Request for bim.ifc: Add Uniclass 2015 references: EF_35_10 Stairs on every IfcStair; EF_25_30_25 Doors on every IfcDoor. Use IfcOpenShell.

First a look at what the model holds.

```python
import ifcopenshell

model = ifcopenshell.open("bim.ifc")
print(model.schema)
print("classifications:", [c.Name for c in model.by_type("IfcClassification")])
for ifc_class in ("IfcDoor", "IfcRoof", "IfcStair", "IfcWall", "IfcWindow"):
    print(ifc_class, len(model.by_type(ifc_class)))
```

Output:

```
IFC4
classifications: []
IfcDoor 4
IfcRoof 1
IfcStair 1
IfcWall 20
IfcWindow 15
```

```python
import ifcopenshell
import ifcopenshell.api.classification

model = ifcopenshell.open("bim.ifc")

system = ifcopenshell.api.classification.add_classification(model, classification="Uniclass 2015")

codes = {
    "IfcStair": ("EF_35_10", "Stairs"),
    "IfcDoor": ("EF_25_30_25", "Doors"),
}
for ifc_class, (code, name) in codes.items():
    products = model.by_type(ifc_class)
    ifcopenshell.api.classification.add_reference(
        model, products=products, classification=system, identification=code, name=name
    )
    print(code, len(products))

model.write("bim_v2.ifc")
```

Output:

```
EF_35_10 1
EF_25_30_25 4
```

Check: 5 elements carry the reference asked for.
